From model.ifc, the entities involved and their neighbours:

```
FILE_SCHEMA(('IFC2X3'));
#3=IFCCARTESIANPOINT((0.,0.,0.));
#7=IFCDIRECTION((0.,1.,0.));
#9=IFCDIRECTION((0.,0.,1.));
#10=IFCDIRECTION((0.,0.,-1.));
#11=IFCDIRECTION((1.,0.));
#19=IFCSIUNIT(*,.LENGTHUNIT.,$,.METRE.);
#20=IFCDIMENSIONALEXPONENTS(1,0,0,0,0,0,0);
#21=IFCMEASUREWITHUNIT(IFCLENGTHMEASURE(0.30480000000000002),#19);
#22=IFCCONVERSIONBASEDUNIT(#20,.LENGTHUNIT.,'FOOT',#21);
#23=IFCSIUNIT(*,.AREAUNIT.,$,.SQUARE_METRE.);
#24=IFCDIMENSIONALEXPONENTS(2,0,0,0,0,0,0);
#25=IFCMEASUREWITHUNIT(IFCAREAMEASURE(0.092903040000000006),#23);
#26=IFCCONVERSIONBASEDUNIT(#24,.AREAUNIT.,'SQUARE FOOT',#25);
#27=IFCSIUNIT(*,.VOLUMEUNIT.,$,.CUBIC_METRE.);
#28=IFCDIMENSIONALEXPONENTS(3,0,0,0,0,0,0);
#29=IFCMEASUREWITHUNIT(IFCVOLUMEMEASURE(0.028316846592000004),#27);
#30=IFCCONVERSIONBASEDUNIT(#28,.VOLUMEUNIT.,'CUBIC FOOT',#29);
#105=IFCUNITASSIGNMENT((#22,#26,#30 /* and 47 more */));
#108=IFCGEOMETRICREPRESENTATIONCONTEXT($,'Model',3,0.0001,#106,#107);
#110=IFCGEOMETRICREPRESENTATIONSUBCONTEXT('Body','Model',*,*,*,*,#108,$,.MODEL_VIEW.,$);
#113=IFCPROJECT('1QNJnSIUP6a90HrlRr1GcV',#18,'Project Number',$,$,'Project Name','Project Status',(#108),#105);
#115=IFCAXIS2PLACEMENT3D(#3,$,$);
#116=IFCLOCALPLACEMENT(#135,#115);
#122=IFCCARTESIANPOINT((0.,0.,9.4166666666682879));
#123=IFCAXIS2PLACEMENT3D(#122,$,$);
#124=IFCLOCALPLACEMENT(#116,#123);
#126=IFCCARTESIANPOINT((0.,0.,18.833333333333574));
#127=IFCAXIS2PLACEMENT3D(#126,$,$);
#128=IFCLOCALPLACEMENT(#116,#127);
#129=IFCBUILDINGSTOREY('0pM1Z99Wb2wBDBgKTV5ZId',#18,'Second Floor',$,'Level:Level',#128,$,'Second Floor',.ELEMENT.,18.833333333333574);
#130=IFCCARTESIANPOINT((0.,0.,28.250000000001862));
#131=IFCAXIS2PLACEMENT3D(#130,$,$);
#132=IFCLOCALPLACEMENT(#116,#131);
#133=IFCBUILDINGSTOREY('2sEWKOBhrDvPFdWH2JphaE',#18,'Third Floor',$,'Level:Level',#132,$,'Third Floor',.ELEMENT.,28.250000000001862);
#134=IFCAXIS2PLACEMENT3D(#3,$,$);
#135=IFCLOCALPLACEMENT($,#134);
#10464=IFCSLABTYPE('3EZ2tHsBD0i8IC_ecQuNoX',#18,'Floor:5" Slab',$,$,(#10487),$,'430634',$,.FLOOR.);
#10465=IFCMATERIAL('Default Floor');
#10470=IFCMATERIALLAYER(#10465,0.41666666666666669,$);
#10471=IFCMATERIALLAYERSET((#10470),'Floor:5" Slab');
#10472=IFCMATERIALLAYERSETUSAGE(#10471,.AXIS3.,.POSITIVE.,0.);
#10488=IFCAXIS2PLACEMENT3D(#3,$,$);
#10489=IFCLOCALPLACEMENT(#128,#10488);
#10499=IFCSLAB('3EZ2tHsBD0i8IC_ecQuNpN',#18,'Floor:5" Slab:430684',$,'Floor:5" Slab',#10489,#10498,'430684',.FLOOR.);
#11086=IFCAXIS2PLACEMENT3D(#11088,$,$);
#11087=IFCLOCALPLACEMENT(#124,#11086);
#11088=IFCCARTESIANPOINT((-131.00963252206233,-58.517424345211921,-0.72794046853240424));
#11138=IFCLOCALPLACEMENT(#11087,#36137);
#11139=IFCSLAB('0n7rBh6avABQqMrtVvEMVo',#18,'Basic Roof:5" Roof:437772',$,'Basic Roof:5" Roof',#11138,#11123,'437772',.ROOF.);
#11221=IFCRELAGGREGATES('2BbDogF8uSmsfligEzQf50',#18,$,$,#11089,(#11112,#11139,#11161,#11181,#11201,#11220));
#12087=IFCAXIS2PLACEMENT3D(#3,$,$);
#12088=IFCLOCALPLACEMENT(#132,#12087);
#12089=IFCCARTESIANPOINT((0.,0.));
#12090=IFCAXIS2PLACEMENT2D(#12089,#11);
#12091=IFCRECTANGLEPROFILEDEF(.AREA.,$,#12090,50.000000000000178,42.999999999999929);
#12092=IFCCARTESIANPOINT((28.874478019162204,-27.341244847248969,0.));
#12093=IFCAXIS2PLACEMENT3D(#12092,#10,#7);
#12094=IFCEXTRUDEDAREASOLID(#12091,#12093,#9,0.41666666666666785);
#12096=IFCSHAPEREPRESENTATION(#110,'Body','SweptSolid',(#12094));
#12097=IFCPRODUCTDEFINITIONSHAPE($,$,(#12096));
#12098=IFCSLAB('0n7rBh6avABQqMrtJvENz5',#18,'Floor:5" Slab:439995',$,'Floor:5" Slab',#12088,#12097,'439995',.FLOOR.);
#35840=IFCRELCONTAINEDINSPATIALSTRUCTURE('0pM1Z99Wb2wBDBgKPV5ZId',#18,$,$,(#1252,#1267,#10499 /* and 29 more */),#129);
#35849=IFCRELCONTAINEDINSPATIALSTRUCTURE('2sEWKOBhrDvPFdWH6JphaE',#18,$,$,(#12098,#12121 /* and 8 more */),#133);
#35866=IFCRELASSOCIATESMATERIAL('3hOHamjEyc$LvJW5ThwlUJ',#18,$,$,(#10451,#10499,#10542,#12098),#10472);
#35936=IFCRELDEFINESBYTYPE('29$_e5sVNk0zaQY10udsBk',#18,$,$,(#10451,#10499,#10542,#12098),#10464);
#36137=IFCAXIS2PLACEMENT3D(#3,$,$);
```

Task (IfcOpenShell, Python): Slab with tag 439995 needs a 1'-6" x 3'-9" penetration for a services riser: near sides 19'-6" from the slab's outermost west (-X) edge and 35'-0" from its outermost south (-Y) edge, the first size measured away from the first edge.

```python
import numpy as np
import ifcopenshell
import ifcopenshell.api.feature
import ifcopenshell.api.geometry
import ifcopenshell.api.root
import ifcopenshell.geom
import ifcopenshell.util.placement
import ifcopenshell.util.representation
import ifcopenshell.util.shape
import ifcopenshell.util.unit

model = ifcopenshell.open("model.ifc")
unit_scale = ifcopenshell.util.unit.calculate_unit_scale(model)
settings = ifcopenshell.geom.settings()


def volume(element):
    """Net volume in cubic metres, openings subtracted."""
    shape = ifcopenshell.geom.create_shape(settings, element)
    return ifcopenshell.util.shape.get_volume(shape.geometry)


slab = model.by_guid("0n7rBh6avABQqMrtJvENz5")
before = volume(slab)

# Extent in the slab's own axes, in metres. The edges named are its -X and -Y sides.
slab_shape = ifcopenshell.geom.create_shape(settings, slab)
vertices = ifcopenshell.util.shape.get_vertices(slab_shape.geometry)
x_min, y_min, bottom = vertices.min(axis=0)
top = vertices[:, 2].max()

opening = ifcopenshell.api.root.create_entity(model, ifc_class="IfcOpeningElement", name="Services riser opening")
context = ifcopenshell.util.representation.get_context(model, "Model", "Body", "MODEL_VIEW")
width, depth = 0.4572, 1.143
outline = [(0.0, 0.0), (width, 0.0), (width, depth), (0.0, depth), (0.0, 0.0)]
# Overshoot both faces by 50 mm so the cut is clean.
shape = ifcopenshell.api.geometry.add_slab_representation(
    model, context=context, depth=top - bottom + 0.1, polyline=outline
)
ifcopenshell.api.geometry.assign_representation(model, product=opening, representation=shape)

matrix = ifcopenshell.util.placement.get_local_placement(slab.ObjectPlacement)
matrix[:, 3] = matrix @ np.append(np.array([x_min + 5.9436, y_min + 10.668, bottom - 0.05]) / unit_scale, 1.0)
ifcopenshell.api.geometry.edit_object_placement(model, product=opening, matrix=matrix, is_si=False)
ifcopenshell.api.feature.add_feature(model, feature=opening, element=slab)

after = volume(slab)

print(f"slab volume {before:.3f} -> {after:.3f} m3")

model.write("model_rev.ifc")
```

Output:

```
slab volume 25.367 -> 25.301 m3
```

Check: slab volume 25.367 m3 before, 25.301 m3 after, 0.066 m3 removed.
